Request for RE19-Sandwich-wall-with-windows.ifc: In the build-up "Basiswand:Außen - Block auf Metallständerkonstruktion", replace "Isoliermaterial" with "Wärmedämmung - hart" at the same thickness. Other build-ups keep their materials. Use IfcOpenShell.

First a look at what the model holds.

```python
import ifcopenshell
import ifcopenshell.util.element

model = ifcopenshell.open("RE19-Sandwich-wall-with-windows.ifc")
print(model.schema)
for layer_set in model.by_type("IfcMaterialLayerSet"):
    if layer_set.LayerSetName == "Basiswand:Außen - Block auf Metallständerkonstruktion":
        for layer in layer_set.MaterialLayers:
            print(layer.id(), layer.Material and layer.Material.Name, layer.LayerThickness, sep=" | ")
        print(len(ifcopenshell.util.element.get_elements_by_material(model, layer_set)), "elements and types use it")
print(sorted(m.Name for m in model.by_type("IfcMaterial") if m.Name)[:60])
```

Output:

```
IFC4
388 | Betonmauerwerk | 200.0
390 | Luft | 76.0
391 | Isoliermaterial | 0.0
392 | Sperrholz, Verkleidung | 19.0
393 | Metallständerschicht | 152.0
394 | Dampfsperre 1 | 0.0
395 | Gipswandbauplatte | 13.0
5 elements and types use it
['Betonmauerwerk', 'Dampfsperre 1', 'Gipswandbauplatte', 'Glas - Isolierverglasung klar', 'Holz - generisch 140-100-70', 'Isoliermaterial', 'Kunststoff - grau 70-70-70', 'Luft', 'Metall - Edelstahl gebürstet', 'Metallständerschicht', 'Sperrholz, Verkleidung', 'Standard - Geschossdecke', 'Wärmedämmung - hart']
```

```python
import ifcopenshell
import ifcopenshell.api.material

model = ifcopenshell.open("RE19-Sandwich-wall-with-windows.ifc")

layer_set = next(s for s in model.by_type("IfcMaterialLayerSet") if s.LayerSetName == "Basiswand:Außen - Block auf Metallständerkonstruktion")
layer = next(l for l in layer_set.MaterialLayers if l.Material and l.Material.Name == "Isoliermaterial")
material = next(m for m in model.by_type("IfcMaterial") if m.Name == "Wärmedämmung - hart")

# Point this one layer at the other material; renaming the old one would change it everywhere.
ifcopenshell.api.material.edit_layer(model, layer=layer, attributes={}, material=material)

print([l.Material.Name if l.Material else None for l in layer_set.MaterialLayers])

model.write("RE19-Sandwich-wall-with-windows_v2.ifc")
```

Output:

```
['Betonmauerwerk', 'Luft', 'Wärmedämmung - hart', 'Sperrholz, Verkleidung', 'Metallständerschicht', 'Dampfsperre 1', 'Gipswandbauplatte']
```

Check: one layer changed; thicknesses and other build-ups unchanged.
